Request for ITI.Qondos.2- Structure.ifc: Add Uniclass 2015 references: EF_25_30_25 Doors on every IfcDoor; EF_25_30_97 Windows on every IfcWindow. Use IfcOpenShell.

First a look at what the model holds.

```python
import ifcopenshell

model = ifcopenshell.open("ITI.Qondos.2- Structure.ifc")
print(model.schema)
print("classifications:", [c.Name for c in model.by_type("IfcClassification")])
for ifc_class in ("IfcDoor", "IfcRoof", "IfcStair", "IfcWall", "IfcWindow"):
    print(ifc_class, len(model.by_type(ifc_class)))
```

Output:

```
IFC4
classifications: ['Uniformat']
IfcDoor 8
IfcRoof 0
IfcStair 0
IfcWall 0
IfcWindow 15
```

```python
import ifcopenshell
import ifcopenshell.api.classification

model = ifcopenshell.open("ITI.Qondos.2- Structure.ifc")

system = ifcopenshell.api.classification.add_classification(model, classification="Uniclass 2015")

codes = {
    "IfcDoor": ("EF_25_30_25", "Doors"),
    "IfcWindow": ("EF_25_30_97", "Windows"),
}
for ifc_class, (code, name) in codes.items():
    products = model.by_type(ifc_class)
    ifcopenshell.api.classification.add_reference(
        model, products=products, classification=system, identification=code, name=name
    )
    print(code, len(products))

model.write("ITI.Qondos.2- Structure_v2.ifc")
```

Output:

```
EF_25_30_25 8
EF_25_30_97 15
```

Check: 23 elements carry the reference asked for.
